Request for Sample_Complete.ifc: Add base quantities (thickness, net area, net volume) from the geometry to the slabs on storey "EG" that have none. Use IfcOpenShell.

First a look at what the model holds.

```python
import ifcopenshell
import ifcopenshell.util.element
import ifcopenshell.util.unit

model = ifcopenshell.open("Sample_Complete.ifc")
print(model.schema)
for unit_type in ("LENGTHUNIT", "AREAUNIT", "VOLUMEUNIT"):
    print(unit_type, ifcopenshell.util.unit.calculate_unit_scale(model, unit_type))
storey = next(s for s in model.by_type("IfcBuildingStorey") if s.Name == "EG")
slabs = [e for e in ifcopenshell.util.element.get_decomposition(storey) if e.is_a("IfcSlab")]
for e in sorted(slabs, key=lambda e: e.id()):
    print(e.id(), e.is_a(), e.Name, list(ifcopenshell.util.element.get_psets(e, qtos_only=True)), sep=" | ")
```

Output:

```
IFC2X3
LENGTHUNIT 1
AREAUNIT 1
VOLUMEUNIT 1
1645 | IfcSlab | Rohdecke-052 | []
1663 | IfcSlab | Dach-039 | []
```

```python
import ifcopenshell
import ifcopenshell.api.pset
import ifcopenshell.geom
import ifcopenshell.util.element
import ifcopenshell.util.shape
import ifcopenshell.util.unit

model = ifcopenshell.open("Sample_Complete.ifc")
unit_scale = ifcopenshell.util.unit.calculate_unit_scale(model)
area_scale = ifcopenshell.util.unit.calculate_unit_scale(model, "AREAUNIT")
volume_scale = ifcopenshell.util.unit.calculate_unit_scale(model, "VOLUMEUNIT")
settings = ifcopenshell.geom.settings()

storey = next(s for s in model.by_type("IfcBuildingStorey") if s.Name == "EG")
slabs = [e for e in ifcopenshell.util.element.get_decomposition(storey) if e.is_a("IfcSlab")]

for e in sorted(slabs, key=lambda e: e.id()):
    if ifcopenshell.util.element.get_psets(e, qtos_only=True, should_inherit=False):
        continue
    # Geometry comes back in metres, in the element's own axes.
    shape = ifcopenshell.geom.create_shape(settings, e)
    values = {
        "Width": ifcopenshell.util.shape.get_z(shape.geometry) / unit_scale,
        "NetArea": ifcopenshell.util.shape.get_footprint_area(shape.geometry) / area_scale,
        "NetVolume": ifcopenshell.util.shape.get_volume(shape.geometry) / volume_scale,
    }
    qto = ifcopenshell.api.pset.add_qto(model, product=e, name="BaseQuantities")
    ifcopenshell.api.pset.edit_qto(model, qto=qto, properties=values)
    print(e.id(), {k: round(v, 3) for k, v in values.items()})

model.write("Sample_Complete_updated.ifc")
```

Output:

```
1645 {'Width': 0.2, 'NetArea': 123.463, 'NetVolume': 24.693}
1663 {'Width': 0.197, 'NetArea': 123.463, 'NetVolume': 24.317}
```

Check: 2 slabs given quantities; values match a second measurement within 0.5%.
